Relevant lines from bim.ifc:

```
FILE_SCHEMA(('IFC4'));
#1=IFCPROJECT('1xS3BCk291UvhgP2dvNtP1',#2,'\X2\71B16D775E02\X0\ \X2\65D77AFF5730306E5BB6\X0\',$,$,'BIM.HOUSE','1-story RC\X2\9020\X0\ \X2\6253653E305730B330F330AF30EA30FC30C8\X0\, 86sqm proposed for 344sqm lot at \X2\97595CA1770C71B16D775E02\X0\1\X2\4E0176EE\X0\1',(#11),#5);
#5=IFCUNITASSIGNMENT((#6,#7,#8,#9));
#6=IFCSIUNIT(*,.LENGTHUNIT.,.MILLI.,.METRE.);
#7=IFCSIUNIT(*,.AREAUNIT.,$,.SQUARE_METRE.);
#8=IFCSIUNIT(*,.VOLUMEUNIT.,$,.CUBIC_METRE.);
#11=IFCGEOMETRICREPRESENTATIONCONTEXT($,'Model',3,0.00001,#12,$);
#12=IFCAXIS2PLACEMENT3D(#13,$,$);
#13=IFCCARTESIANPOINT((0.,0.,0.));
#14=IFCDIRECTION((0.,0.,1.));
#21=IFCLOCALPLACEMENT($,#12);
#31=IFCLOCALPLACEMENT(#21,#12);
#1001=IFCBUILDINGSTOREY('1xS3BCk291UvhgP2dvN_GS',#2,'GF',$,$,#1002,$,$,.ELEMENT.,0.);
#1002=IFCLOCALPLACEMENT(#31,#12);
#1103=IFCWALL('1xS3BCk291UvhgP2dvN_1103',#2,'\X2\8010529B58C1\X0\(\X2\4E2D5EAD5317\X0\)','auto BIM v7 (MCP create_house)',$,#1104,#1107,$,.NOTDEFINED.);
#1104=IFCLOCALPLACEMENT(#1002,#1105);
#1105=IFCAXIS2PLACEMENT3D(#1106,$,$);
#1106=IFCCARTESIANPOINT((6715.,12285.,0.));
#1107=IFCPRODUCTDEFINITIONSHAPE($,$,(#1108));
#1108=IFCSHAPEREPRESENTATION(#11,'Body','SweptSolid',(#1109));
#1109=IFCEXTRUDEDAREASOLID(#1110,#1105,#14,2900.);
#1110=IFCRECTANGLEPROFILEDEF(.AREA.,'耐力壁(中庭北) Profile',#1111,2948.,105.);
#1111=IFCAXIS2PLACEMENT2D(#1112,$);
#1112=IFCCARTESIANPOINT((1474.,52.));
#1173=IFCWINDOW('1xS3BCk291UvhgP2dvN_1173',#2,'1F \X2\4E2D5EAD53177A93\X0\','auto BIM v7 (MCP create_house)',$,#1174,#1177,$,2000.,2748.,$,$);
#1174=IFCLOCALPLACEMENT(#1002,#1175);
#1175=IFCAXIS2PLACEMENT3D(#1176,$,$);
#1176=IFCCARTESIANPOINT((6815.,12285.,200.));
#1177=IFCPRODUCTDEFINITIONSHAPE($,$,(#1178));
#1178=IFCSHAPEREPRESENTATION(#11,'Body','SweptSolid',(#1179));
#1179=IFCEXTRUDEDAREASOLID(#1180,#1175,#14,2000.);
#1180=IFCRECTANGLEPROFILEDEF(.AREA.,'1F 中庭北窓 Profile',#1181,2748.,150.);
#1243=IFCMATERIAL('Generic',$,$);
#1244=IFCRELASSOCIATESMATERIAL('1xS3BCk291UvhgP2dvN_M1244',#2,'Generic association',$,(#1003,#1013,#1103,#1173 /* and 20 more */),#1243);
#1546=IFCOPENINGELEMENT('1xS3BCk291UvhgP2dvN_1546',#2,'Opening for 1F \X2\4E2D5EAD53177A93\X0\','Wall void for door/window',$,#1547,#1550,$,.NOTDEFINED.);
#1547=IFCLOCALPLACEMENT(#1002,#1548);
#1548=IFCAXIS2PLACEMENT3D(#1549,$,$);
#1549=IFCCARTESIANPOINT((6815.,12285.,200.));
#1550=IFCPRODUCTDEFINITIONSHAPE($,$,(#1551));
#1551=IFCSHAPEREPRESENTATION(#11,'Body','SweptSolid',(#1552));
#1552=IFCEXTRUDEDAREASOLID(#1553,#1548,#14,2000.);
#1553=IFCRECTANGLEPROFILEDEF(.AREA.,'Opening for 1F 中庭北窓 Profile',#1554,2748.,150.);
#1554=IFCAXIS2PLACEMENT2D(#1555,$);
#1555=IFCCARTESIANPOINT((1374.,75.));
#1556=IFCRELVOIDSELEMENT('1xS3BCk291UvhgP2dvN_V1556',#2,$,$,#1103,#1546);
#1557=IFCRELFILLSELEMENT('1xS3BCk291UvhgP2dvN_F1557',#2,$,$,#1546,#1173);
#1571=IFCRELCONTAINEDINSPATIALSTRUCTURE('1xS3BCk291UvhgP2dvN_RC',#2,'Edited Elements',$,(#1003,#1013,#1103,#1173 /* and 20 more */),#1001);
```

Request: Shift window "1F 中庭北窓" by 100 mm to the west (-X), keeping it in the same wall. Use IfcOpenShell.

```python
import ifcopenshell
import ifcopenshell.api.geometry
import ifcopenshell.util.placement
import ifcopenshell.util.unit

model = ifcopenshell.open("bim.ifc")
unit_scale = ifcopenshell.util.unit.calculate_unit_scale(model)

window = model.by_id(1173)
opening = window.FillsVoids[0].RelatingOpeningElement
wall = opening.VoidsElements[0].RelatingBuildingElement

wall_matrix = ifcopenshell.util.placement.get_local_placement(wall.ObjectPlacement)
shift = wall_matrix[:3, 0] * -0.1 / unit_scale
before = ifcopenshell.util.placement.get_local_placement(window.ObjectPlacement)[:3, 3].copy()

# The window is not placed relative to its opening, so move both.
for product in (opening, window):
    matrix = ifcopenshell.util.placement.get_local_placement(product.ObjectPlacement)
    matrix[:3, 3] += shift
    ifcopenshell.api.geometry.edit_object_placement(model, product=product, matrix=matrix, is_si=False)

after = ifcopenshell.util.placement.get_local_placement(window.ObjectPlacement)[:3, 3]
print("window moved by", (after - before).round(3) + 0.0)

model.write("bim_v2.ifc")
```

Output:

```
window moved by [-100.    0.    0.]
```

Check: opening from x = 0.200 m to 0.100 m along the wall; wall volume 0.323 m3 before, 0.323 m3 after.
